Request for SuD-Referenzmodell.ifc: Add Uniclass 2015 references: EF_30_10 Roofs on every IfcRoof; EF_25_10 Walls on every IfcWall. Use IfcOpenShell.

First a look at what the model holds.

```python
import ifcopenshell

model = ifcopenshell.open("SuD-Referenzmodell.ifc")
print(model.schema)
print("classifications:", [c.Name for c in model.by_type("IfcClassification")])
for ifc_class in ("IfcDoor", "IfcRoof", "IfcStair", "IfcWall", "IfcWindow"):
    print(ifc_class, len(model.by_type(ifc_class)))
```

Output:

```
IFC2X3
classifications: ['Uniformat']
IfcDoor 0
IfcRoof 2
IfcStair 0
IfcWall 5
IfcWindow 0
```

```python
import ifcopenshell
import ifcopenshell.api.classification

model = ifcopenshell.open("SuD-Referenzmodell.ifc")

# IFC2X3 requires Source and Edition and has no link from the project to the system.
system = model.create_entity("IfcClassification", Source="NBS", Edition="2015", Name="Uniclass 2015")

codes = {
    "IfcRoof": ("EF_30_10", "Roofs"),
    "IfcWall": ("EF_25_10", "Walls"),
}
for ifc_class, (code, name) in codes.items():
    products = model.by_type(ifc_class)
    ifcopenshell.api.classification.add_reference(
        model, products=products, classification=system, identification=code, name=name
    )
    print(code, len(products))

model.write("SuD-Referenzmodell_edited.ifc")
```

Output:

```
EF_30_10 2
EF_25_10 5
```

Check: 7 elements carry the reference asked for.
